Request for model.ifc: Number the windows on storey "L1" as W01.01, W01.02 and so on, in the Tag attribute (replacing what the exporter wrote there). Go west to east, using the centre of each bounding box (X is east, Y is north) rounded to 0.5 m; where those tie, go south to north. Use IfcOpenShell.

First a look at what the model holds.

```python
import ifcopenshell
import ifcopenshell.util.element
import ifcopenshell.util.placement

model = ifcopenshell.open("model.ifc")
print(model.schema)
storey = next(s for s in model.by_type("IfcBuildingStorey") if s.Name == "L1")
windows = [e for e in ifcopenshell.util.element.get_decomposition(storey) if e.is_a("IfcWindow")]
for e in sorted(windows, key=lambda e: e.id()):
    origin = ifcopenshell.util.placement.get_local_placement(e.ObjectPlacement)[:3, 3]
    print(e.id(), e.Tag, e.Name, origin.round(2) + 0.0, sep=" | ")
```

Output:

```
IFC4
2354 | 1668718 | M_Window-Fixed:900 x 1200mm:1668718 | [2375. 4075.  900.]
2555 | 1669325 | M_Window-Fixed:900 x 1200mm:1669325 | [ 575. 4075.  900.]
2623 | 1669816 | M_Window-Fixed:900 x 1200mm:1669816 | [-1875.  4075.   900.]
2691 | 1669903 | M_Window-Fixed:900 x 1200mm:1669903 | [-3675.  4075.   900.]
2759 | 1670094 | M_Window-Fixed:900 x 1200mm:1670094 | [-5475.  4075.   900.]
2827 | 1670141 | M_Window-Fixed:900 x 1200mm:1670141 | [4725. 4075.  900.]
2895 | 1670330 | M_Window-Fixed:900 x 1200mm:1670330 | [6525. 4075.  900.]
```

```python
import ifcopenshell
import ifcopenshell.geom
import ifcopenshell.util.element
import ifcopenshell.util.shape

model = ifcopenshell.open("model.ifc")
settings = ifcopenshell.geom.settings()
settings.set("use-world-coords", True)


def centre(element):
    shape = ifcopenshell.geom.create_shape(settings, element)
    return ifcopenshell.util.shape.get_bbox_centroid(shape.geometry)


storey = next(s for s in model.by_type("IfcBuildingStorey") if s.Name == "L1")
windows = [e for e in ifcopenshell.util.element.get_decomposition(storey) if e.is_a("IfcWindow")]

# Insertion points can sit at a corner or the storey origin, so sort by the geometry (in metres).
centres = {e: centre(e) for e in windows}
windows.sort(key=lambda e: (round(centres[e][0] / 0.5), centres[e][1]))

for i, e in enumerate(windows, start=1):
    number = f"W01.{i:02d}"
    e.Tag = number
    print(e.id(), number)

model.write("model_rev.ifc")
```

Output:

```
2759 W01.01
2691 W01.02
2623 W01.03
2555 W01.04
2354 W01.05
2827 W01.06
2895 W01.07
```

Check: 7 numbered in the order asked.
